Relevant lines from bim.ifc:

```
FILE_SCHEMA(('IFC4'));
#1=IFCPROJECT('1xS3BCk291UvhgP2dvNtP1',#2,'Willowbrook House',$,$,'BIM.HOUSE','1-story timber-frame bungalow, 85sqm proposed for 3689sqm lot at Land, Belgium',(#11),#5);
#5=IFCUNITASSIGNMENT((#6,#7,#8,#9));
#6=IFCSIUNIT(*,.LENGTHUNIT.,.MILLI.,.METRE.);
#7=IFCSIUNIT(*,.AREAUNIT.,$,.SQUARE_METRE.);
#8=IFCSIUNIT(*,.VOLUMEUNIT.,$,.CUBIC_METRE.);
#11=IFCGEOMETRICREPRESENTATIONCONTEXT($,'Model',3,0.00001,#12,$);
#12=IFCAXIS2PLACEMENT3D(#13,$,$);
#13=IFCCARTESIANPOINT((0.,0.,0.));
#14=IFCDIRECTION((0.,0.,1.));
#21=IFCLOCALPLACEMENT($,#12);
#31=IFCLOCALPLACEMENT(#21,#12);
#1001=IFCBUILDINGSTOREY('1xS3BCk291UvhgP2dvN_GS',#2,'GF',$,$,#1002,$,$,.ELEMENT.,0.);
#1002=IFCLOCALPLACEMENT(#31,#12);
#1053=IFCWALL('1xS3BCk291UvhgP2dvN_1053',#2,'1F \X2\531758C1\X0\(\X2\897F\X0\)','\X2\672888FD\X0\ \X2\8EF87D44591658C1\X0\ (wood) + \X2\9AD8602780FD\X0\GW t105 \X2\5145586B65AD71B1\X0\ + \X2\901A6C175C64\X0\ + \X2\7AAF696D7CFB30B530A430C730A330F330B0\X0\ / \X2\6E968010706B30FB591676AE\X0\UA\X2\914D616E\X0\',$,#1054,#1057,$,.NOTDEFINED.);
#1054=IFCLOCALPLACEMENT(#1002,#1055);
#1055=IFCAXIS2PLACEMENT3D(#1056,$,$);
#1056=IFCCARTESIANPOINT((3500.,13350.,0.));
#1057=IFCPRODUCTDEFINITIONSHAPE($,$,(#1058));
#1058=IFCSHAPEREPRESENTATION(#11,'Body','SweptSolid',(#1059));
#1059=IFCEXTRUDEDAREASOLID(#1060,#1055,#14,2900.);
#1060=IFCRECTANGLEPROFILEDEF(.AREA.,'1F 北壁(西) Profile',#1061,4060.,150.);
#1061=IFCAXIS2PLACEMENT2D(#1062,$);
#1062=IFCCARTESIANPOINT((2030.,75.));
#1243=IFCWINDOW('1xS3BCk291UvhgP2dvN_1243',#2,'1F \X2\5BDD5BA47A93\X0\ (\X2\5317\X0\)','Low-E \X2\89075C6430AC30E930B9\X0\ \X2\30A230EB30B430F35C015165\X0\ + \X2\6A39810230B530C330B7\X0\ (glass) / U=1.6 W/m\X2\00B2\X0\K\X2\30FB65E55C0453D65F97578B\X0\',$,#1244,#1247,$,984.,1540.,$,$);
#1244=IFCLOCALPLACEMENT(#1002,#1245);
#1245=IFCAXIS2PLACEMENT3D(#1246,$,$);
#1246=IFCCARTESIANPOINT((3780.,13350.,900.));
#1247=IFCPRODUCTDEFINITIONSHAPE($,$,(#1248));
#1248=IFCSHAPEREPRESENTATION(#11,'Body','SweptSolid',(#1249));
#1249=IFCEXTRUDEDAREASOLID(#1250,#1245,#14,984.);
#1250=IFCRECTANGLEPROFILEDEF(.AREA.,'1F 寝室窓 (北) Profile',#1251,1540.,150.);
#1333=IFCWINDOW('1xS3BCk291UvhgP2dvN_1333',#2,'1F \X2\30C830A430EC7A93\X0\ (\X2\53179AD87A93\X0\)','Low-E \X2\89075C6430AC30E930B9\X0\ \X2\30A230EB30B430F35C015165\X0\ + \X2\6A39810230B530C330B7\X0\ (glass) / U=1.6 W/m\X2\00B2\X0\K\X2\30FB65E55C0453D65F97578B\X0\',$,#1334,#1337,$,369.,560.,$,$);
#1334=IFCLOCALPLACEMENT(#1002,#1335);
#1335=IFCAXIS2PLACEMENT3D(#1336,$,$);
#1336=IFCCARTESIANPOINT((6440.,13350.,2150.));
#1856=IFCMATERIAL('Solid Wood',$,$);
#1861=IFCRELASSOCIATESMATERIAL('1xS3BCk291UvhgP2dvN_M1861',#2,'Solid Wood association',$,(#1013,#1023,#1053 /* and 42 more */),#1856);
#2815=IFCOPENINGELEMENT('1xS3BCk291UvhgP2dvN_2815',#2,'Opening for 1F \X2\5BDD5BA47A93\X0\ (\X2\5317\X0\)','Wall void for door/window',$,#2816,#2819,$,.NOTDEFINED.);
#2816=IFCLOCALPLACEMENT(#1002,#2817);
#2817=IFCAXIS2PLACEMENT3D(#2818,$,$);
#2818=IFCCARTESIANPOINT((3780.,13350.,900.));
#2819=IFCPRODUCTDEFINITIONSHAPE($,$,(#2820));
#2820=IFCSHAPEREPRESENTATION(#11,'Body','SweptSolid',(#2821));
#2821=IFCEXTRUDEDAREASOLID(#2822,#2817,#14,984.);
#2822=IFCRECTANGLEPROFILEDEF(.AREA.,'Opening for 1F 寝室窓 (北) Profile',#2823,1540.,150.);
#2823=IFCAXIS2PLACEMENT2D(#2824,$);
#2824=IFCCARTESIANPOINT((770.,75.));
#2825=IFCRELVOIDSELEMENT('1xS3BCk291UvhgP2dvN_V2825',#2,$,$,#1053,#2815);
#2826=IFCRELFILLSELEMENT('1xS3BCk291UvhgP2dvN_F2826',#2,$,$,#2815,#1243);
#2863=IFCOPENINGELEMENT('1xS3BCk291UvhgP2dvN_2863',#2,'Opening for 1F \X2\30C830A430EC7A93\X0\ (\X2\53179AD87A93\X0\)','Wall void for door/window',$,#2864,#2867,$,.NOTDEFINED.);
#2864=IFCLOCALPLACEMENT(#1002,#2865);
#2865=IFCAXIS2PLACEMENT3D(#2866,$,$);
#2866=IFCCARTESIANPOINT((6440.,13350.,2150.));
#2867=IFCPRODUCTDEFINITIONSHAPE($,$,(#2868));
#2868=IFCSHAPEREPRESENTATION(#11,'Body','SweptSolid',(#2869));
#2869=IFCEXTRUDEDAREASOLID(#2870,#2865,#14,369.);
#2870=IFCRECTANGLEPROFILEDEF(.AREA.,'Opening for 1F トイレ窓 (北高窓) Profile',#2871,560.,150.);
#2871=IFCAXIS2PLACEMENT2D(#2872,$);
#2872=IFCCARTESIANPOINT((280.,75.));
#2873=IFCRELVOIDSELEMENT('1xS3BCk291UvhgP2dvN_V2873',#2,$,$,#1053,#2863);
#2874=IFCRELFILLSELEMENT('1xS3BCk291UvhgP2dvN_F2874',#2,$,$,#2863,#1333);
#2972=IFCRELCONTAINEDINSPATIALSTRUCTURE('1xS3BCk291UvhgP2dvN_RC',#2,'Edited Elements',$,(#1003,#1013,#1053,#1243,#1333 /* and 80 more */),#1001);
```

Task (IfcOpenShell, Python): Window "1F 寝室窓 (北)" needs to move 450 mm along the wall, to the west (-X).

```python
import ifcopenshell
import ifcopenshell.api.geometry
import ifcopenshell.util.placement
import ifcopenshell.util.unit

model = ifcopenshell.open("bim.ifc")
unit_scale = ifcopenshell.util.unit.calculate_unit_scale(model)

window = model.by_guid("1xS3BCk291UvhgP2dvN_1243")
opening = window.FillsVoids[0].RelatingOpeningElement
wall = opening.VoidsElements[0].RelatingBuildingElement

wall_matrix = ifcopenshell.util.placement.get_local_placement(wall.ObjectPlacement)
shift = wall_matrix[:3, 0] * -0.45 / unit_scale
before = ifcopenshell.util.placement.get_local_placement(window.ObjectPlacement)[:3, 3].copy()

# The window is not placed relative to its opening, so move both.
for product in (opening, window):
    matrix = ifcopenshell.util.placement.get_local_placement(product.ObjectPlacement)
    matrix[:3, 3] += shift
    ifcopenshell.api.geometry.edit_object_placement(model, product=product, matrix=matrix, is_si=False)

after = ifcopenshell.util.placement.get_local_placement(window.ObjectPlacement)[:3, 3]
print("window moved by", (after - before).round(3) + 0.0)

model.write("bim_edited.ifc")
```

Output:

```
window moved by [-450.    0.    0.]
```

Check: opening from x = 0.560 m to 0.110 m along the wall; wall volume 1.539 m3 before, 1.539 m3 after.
